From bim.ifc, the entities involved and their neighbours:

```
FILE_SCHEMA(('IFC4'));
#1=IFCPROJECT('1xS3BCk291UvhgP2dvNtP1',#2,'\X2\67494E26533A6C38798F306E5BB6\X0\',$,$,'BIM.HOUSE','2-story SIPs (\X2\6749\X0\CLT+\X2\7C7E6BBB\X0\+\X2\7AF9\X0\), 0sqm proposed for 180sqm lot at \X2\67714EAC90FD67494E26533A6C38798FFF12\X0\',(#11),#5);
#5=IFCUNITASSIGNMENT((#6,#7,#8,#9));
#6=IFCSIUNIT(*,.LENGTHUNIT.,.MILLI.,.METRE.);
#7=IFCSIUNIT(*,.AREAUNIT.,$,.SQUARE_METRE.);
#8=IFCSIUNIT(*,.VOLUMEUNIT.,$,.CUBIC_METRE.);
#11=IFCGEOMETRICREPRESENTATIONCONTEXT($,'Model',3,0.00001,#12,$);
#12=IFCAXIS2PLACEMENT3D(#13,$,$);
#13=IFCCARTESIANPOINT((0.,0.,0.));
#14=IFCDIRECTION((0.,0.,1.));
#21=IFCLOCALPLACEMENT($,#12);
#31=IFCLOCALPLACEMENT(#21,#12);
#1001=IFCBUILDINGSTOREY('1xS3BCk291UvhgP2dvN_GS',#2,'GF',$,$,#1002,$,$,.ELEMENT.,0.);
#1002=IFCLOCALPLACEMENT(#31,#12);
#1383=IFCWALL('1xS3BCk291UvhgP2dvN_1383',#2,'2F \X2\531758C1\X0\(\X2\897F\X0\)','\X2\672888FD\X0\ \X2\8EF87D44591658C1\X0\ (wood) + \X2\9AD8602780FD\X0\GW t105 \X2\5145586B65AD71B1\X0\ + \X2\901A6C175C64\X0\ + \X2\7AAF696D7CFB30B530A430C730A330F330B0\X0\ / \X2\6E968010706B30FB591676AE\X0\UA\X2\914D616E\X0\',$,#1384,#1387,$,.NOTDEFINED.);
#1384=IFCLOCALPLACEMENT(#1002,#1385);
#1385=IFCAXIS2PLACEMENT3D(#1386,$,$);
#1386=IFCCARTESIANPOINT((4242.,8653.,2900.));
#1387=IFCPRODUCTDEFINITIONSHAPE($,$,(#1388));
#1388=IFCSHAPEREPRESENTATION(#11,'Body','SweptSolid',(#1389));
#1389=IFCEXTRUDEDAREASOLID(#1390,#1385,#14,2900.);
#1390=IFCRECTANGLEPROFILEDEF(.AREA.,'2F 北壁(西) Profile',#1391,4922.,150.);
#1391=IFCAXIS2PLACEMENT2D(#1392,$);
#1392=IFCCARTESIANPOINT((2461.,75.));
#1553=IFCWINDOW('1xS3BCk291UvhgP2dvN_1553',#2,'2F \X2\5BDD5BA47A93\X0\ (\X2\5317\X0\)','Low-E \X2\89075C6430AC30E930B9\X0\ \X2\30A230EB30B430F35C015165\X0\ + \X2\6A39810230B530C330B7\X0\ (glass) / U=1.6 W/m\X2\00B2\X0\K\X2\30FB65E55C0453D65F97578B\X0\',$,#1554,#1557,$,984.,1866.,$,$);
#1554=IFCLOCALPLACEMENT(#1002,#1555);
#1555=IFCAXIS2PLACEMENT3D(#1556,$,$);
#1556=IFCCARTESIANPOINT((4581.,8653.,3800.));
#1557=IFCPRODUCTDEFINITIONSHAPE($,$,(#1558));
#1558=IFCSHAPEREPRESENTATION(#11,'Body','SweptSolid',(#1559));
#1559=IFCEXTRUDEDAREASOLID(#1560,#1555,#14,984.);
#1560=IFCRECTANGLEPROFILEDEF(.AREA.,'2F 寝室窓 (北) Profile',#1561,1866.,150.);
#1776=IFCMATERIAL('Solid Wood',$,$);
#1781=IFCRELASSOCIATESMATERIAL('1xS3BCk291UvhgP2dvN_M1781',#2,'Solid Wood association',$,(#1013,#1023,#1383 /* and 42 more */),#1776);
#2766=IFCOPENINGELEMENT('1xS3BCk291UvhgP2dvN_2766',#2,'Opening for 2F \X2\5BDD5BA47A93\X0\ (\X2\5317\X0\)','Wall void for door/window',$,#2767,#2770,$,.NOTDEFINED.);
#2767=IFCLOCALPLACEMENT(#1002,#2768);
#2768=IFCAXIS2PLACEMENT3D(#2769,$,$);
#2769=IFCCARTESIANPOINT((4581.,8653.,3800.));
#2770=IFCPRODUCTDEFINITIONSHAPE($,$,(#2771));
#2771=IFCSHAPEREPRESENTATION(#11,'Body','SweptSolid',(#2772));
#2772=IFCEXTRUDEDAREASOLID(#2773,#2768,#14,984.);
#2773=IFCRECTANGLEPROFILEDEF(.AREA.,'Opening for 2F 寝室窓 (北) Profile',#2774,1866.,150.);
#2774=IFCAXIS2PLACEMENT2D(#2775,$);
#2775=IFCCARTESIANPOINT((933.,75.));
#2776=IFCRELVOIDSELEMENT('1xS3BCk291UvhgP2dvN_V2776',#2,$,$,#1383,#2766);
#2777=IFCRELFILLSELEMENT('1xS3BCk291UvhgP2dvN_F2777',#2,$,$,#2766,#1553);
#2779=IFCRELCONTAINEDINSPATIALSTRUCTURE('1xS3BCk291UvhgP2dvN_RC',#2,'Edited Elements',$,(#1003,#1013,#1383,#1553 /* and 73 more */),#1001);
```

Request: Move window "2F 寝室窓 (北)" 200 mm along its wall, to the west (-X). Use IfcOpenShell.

```python
import ifcopenshell
import ifcopenshell.api.geometry
import ifcopenshell.util.placement
import ifcopenshell.util.unit

model = ifcopenshell.open("bim.ifc")
unit_scale = ifcopenshell.util.unit.calculate_unit_scale(model)

window = model.by_guid("1xS3BCk291UvhgP2dvN_1553")
opening = window.FillsVoids[0].RelatingOpeningElement
wall = opening.VoidsElements[0].RelatingBuildingElement

wall_matrix = ifcopenshell.util.placement.get_local_placement(wall.ObjectPlacement)
shift = wall_matrix[:3, 0] * -0.2 / unit_scale
before = ifcopenshell.util.placement.get_local_placement(window.ObjectPlacement)[:3, 3].copy()

# The window is not placed relative to its opening, so move both.
for product in (opening, window):
    matrix = ifcopenshell.util.placement.get_local_placement(product.ObjectPlacement)
    matrix[:3, 3] += shift
    ifcopenshell.api.geometry.edit_object_placement(model, product=product, matrix=matrix, is_si=False)

after = ifcopenshell.util.placement.get_local_placement(window.ObjectPlacement)[:3, 3]
print("window moved by", (after - before).round(3) + 0.0)

model.write("bim_rev.ifc")
```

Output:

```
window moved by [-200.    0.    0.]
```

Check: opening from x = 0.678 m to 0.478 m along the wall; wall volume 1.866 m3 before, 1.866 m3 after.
